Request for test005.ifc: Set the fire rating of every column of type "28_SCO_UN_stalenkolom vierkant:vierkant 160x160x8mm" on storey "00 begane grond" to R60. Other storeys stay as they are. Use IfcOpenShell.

First a look at what the model holds.

```python
import ifcopenshell
import ifcopenshell.util.element

model = ifcopenshell.open("test005.ifc")
print(model.schema)
storey = next(s for s in model.by_type("IfcBuildingStorey") if s.Name == "00 begane grond")
columns = [e for e in ifcopenshell.util.element.get_decomposition(storey) if e.is_a("IfcColumn")]
seen = {}
for e in columns:
    element_type = ifcopenshell.util.element.get_type(e)
    key = (element_type.Name if element_type != e and element_type else None, ifcopenshell.util.element.get_pset(e, "Pset_ColumnCommon", "FireRating"))
    seen[key] = seen.get(key, 0) + 1
for (name, value), count in sorted(seen.items(), key=str):
    print(count, "x", name, "|", value)
```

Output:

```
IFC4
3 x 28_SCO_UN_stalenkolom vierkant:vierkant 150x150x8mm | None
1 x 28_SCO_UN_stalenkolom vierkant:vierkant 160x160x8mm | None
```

```python
import ifcopenshell
import ifcopenshell.api.pset
import ifcopenshell.util.element

model = ifcopenshell.open("test005.ifc")

storey = next(s for s in model.by_type("IfcBuildingStorey") if s.Name == "00 begane grond")
columns = [e for e in ifcopenshell.util.element.get_decomposition(storey) if e.is_a("IfcColumn")]

count = 0
for e in columns:
    element_type = ifcopenshell.util.element.get_type(e)
    if element_type in (None, e) or element_type.Name != "28_SCO_UN_stalenkolom vierkant:vierkant 160x160x8mm":
        continue
    # add_pset returns the element's existing set when there is one.
    pset = ifcopenshell.api.pset.add_pset(model, product=e, name="Pset_ColumnCommon")
    ifcopenshell.api.pset.edit_pset(model, pset=pset, properties={"FireRating": "R60"})
    count += 1

print(count, "columns updated")

model.write("test005_updated.ifc")
```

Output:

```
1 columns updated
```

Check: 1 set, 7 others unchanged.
